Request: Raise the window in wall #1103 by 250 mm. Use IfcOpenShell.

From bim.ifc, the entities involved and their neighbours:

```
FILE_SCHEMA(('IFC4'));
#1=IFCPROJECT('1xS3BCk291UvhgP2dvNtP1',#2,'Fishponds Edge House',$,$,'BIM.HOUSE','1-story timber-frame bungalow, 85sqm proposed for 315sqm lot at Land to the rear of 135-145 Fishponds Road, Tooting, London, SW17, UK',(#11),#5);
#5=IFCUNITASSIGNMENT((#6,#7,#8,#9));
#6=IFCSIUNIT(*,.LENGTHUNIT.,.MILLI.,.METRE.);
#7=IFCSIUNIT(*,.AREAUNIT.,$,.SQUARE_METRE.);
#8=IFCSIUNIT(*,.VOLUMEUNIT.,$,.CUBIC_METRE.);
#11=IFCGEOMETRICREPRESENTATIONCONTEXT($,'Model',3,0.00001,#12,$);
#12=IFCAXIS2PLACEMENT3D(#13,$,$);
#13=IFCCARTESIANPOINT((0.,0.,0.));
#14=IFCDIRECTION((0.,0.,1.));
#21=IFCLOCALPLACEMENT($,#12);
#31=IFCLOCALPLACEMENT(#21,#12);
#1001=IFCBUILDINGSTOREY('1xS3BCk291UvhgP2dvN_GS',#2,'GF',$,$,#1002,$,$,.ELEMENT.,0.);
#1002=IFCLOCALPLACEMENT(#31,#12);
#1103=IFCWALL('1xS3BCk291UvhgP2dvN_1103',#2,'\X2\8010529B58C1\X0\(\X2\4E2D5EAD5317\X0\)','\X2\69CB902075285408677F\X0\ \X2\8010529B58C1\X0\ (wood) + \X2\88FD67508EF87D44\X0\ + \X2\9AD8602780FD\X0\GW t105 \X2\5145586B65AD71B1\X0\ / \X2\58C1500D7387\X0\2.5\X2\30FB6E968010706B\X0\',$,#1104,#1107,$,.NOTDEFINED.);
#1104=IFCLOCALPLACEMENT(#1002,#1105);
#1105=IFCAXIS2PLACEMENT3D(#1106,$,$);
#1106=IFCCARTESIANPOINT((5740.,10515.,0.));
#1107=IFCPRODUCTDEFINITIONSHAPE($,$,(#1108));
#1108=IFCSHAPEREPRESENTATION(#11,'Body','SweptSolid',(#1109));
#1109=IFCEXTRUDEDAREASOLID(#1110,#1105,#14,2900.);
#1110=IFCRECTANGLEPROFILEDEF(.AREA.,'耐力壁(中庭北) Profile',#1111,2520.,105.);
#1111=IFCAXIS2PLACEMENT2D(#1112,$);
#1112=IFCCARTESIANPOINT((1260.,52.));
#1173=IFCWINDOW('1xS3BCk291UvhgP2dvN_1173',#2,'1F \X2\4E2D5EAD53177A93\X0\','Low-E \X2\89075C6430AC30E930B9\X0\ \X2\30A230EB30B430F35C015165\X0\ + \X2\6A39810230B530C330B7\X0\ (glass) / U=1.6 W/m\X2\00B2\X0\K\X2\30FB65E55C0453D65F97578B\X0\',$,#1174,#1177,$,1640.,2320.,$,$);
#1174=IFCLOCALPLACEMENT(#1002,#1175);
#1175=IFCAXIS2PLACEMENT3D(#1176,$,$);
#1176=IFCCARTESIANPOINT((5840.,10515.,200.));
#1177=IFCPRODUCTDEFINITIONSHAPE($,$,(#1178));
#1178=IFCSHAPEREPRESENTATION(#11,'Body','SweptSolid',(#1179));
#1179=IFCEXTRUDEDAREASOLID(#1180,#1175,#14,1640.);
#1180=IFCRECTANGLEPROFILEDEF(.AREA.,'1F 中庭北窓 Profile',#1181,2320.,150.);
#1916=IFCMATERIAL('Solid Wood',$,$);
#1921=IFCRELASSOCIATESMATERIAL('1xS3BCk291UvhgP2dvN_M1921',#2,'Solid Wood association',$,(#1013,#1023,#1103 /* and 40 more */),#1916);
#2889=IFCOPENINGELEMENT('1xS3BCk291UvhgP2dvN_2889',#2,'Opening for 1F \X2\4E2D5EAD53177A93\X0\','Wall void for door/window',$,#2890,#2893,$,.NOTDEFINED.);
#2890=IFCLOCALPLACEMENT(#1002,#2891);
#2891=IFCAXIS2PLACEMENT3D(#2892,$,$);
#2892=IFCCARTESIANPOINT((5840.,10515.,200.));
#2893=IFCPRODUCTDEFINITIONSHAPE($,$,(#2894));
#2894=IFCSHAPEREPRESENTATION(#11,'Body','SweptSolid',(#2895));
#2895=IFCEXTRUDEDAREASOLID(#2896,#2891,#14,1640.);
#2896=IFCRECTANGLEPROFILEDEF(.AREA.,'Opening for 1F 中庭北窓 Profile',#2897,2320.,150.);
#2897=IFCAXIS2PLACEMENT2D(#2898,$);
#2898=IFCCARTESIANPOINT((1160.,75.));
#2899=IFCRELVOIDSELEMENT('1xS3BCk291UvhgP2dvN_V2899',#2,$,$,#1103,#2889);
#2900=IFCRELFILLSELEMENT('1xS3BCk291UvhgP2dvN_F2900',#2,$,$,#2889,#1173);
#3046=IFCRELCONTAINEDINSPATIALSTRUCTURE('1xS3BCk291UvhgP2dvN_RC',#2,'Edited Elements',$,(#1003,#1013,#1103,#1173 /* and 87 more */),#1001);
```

```python
import numpy as np
import ifcopenshell
import ifcopenshell.api.geometry
import ifcopenshell.util.placement
import ifcopenshell.util.unit

model = ifcopenshell.open("bim.ifc")
unit_scale = ifcopenshell.util.unit.calculate_unit_scale(model)

window = model.by_guid("1xS3BCk291UvhgP2dvN_1173")
opening = window.FillsVoids[0].RelatingOpeningElement
dz = 0.25 / unit_scale

shift = np.array([0.0, 0.0, dz])
# The window is not placed relative to its opening, so move both.
for product in (opening, window):
    matrix = ifcopenshell.util.placement.get_local_placement(product.ObjectPlacement)
    matrix[:3, 3] += shift
    ifcopenshell.api.geometry.edit_object_placement(model, product=product, matrix=matrix, is_si=False)

print(f"moved by {dz * unit_scale:+.3f} m")

model.write("bim_rev.ifc")
```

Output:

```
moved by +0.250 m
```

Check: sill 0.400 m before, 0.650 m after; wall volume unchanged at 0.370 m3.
